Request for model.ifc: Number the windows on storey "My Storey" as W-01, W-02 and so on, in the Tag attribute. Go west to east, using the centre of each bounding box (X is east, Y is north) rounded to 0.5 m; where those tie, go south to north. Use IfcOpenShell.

First a look at what the model holds.

```python
import ifcopenshell
import ifcopenshell.util.element
import ifcopenshell.util.placement

model = ifcopenshell.open("model.ifc")
print(model.schema)
storey = next(s for s in model.by_type("IfcBuildingStorey") if s.Name == "My Storey")
windows = [e for e in ifcopenshell.util.element.get_decomposition(storey) if e.is_a("IfcWindow")]
for e in sorted(windows, key=lambda e: e.id()):
    origin = ifcopenshell.util.placement.get_local_placement(e.ObjectPlacement)[:3, 3]
    print(e.id(), e.Tag, e.Name, origin.round(2) + 0.0, sep=" | ")
```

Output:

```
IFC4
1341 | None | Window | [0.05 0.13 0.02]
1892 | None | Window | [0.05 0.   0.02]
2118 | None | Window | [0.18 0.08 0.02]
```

```python
import ifcopenshell
import ifcopenshell.geom
import ifcopenshell.util.element
import ifcopenshell.util.shape

model = ifcopenshell.open("model.ifc")
settings = ifcopenshell.geom.settings()
settings.set("use-world-coords", True)


def centre(element):
    shape = ifcopenshell.geom.create_shape(settings, element)
    return ifcopenshell.util.shape.get_bbox_centroid(shape.geometry)


storey = next(s for s in model.by_type("IfcBuildingStorey") if s.Name == "My Storey")
windows = [e for e in ifcopenshell.util.element.get_decomposition(storey) if e.is_a("IfcWindow")]

# Insertion points can sit at a corner or the storey origin, so sort by the geometry (in metres).
centres = {e: centre(e) for e in windows}
windows.sort(key=lambda e: (round(centres[e][0] / 0.5), centres[e][1]))

for i, e in enumerate(windows, start=1):
    number = f"W-{i:02d}"
    e.Tag = number
    print(e.id(), number)

model.write("model_edited.ifc")
```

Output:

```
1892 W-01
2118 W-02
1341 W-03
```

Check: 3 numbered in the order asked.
